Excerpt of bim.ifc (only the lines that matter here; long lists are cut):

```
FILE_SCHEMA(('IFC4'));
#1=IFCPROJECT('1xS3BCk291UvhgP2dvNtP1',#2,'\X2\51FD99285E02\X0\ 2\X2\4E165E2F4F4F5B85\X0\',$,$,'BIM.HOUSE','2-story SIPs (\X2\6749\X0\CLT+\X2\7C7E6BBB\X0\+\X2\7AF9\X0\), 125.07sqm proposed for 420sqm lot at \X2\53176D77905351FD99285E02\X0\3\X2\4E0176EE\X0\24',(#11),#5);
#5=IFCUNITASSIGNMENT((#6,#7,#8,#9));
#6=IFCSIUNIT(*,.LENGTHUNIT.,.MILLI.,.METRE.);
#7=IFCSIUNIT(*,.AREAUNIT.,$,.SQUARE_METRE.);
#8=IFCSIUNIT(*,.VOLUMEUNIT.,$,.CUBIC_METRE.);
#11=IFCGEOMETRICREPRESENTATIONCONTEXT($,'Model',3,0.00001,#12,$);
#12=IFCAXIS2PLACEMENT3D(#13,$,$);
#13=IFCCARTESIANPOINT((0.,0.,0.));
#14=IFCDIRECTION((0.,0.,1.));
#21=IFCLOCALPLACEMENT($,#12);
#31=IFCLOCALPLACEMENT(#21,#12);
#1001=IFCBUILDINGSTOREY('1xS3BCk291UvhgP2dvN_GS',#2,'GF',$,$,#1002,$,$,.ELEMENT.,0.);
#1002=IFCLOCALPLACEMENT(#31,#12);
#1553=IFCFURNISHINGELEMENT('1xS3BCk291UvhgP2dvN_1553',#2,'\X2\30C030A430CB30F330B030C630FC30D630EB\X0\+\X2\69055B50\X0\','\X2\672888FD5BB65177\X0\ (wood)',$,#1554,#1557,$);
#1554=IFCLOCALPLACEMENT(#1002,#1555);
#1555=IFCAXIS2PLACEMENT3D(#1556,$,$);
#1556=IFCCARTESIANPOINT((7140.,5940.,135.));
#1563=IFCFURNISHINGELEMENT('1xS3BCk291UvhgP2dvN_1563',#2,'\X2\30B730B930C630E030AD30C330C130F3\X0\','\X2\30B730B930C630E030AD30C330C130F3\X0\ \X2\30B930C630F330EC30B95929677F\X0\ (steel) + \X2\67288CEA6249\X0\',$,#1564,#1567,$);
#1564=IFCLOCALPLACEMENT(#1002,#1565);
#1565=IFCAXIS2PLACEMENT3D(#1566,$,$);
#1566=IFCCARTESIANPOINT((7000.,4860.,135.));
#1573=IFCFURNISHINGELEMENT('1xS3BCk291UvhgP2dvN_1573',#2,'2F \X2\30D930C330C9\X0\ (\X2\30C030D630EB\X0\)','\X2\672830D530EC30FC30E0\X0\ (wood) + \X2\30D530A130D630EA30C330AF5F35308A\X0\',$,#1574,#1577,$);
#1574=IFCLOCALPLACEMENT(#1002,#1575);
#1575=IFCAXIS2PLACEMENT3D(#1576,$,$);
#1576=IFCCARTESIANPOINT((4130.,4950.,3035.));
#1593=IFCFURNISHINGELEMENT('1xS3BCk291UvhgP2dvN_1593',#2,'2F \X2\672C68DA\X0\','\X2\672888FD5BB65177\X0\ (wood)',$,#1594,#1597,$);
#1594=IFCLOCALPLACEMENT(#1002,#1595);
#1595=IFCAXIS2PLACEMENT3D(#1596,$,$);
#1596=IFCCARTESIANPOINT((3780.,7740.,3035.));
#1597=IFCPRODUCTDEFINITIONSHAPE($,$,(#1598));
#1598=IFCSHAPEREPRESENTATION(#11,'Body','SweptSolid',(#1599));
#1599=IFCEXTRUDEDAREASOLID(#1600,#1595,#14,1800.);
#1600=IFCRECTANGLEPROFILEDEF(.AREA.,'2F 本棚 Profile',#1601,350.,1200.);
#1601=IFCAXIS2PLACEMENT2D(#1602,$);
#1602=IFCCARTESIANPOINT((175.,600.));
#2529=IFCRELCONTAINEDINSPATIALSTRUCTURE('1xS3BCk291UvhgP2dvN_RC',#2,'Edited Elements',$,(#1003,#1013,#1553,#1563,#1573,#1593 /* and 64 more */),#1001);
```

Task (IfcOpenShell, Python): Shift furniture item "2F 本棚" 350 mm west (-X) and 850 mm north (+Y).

```python
import ifcopenshell
import ifcopenshell.api.geometry
import ifcopenshell.util.placement
import ifcopenshell.util.unit

model = ifcopenshell.open("bim.ifc")
unit_scale = ifcopenshell.util.unit.calculate_unit_scale(model)

item = model.by_guid("1xS3BCk291UvhgP2dvN_1593")
matrix = ifcopenshell.util.placement.get_local_placement(item.ObjectPlacement)
matrix[0, 3] -= 0.35 / unit_scale
matrix[1, 3] += 0.85 / unit_scale
ifcopenshell.api.geometry.edit_object_placement(model, product=item, matrix=matrix, is_si=False)

print(ifcopenshell.util.placement.get_local_placement(item.ObjectPlacement).round(3) + 0.0)

model.write("bim_updated.ifc")
```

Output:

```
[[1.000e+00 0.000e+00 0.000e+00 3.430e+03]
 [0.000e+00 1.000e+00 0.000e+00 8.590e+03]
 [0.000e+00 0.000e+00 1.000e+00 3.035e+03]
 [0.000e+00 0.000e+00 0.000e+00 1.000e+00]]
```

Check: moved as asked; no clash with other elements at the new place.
